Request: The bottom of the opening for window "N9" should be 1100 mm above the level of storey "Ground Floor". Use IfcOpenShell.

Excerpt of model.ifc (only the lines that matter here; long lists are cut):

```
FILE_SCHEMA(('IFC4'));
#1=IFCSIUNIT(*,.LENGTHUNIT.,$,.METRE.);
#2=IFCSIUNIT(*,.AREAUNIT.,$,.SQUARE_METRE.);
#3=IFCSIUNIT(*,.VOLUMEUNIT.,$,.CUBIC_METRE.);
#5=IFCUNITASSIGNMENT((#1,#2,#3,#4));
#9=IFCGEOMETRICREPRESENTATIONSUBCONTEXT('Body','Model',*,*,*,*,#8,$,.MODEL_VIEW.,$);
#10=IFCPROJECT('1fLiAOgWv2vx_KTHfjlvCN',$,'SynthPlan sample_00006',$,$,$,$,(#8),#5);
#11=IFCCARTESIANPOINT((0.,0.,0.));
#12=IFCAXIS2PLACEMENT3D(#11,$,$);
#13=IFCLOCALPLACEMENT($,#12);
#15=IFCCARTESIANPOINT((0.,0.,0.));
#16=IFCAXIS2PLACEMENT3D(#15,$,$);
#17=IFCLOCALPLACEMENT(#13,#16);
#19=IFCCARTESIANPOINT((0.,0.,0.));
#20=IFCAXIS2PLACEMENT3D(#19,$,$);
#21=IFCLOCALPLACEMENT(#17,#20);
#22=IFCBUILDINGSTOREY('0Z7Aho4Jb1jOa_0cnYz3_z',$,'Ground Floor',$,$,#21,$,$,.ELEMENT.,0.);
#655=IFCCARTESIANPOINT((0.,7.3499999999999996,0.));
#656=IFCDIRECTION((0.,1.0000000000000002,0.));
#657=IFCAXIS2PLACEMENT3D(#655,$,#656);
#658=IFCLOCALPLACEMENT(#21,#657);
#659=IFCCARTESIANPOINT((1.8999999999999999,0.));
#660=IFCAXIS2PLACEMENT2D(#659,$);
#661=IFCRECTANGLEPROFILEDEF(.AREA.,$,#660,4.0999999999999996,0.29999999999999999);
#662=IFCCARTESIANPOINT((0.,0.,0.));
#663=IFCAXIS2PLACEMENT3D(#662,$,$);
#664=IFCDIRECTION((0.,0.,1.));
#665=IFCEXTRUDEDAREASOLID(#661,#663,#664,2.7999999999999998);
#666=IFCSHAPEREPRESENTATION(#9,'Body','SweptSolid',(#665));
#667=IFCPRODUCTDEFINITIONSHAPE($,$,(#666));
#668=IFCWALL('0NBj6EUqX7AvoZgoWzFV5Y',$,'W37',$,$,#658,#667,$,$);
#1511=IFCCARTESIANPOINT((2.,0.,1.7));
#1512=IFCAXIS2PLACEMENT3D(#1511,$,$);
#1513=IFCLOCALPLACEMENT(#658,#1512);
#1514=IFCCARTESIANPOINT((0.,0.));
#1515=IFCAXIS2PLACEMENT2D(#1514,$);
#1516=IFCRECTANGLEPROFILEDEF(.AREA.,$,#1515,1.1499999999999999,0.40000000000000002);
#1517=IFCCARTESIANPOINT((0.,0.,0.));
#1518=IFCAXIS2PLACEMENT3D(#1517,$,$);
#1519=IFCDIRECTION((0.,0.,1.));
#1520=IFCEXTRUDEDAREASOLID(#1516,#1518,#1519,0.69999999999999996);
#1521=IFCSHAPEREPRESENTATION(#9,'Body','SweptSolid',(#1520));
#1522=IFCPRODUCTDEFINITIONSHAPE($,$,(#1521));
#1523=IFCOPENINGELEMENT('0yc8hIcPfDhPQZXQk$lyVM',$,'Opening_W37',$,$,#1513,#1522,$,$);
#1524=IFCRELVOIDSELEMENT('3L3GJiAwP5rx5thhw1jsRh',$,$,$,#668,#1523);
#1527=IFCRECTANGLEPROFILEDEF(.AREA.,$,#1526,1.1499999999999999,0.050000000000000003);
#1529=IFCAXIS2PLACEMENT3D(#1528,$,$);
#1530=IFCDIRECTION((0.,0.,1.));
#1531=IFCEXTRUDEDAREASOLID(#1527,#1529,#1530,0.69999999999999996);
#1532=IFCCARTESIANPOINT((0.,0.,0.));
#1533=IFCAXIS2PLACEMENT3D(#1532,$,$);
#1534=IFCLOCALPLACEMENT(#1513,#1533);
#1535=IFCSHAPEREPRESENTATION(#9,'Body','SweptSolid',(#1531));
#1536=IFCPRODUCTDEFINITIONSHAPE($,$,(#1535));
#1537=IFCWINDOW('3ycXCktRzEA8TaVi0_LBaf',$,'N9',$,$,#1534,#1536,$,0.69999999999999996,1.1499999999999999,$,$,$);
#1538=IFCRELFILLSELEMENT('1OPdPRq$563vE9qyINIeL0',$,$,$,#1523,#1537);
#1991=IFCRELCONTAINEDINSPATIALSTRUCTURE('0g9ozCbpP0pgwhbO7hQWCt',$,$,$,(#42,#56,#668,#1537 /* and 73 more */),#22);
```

```python
import numpy as np
import ifcopenshell
import ifcopenshell.api.geometry
import ifcopenshell.geom
import ifcopenshell.util.element
import ifcopenshell.util.placement
import ifcopenshell.util.shape
import ifcopenshell.util.unit

model = ifcopenshell.open("model.ifc")
unit_scale = ifcopenshell.util.unit.calculate_unit_scale(model)

window = model.by_guid("3ycXCktRzEA8TaVi0_LBaf")
opening = window.FillsVoids[0].RelatingOpeningElement
storey = ifcopenshell.util.element.get_container(window, ifc_class="IfcBuildingStorey")
level = ifcopenshell.util.placement.get_local_placement(storey.ObjectPlacement)[2, 3]

# The opening's origin need not be at the sill, so measure its lowest point.
shape = ifcopenshell.geom.create_shape(ifcopenshell.geom.settings(), opening)
bottom = ifcopenshell.util.shape.get_shape_bottom_elevation(shape, shape.geometry) / unit_scale
dz = level + 1.1 - bottom

shift = np.array([0.0, 0.0, dz])
# The window is placed relative to its opening, so it follows when the opening moves.
matrix = ifcopenshell.util.placement.get_local_placement(opening.ObjectPlacement)
matrix[:3, 3] += shift
ifcopenshell.api.geometry.edit_object_placement(
    model, product=opening, matrix=matrix, is_si=False, should_transform_children=True
)

print(f"moved by {dz * unit_scale:+.3f} m")

model.write("model_updated.ifc")
```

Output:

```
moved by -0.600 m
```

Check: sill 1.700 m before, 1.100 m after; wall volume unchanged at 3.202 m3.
